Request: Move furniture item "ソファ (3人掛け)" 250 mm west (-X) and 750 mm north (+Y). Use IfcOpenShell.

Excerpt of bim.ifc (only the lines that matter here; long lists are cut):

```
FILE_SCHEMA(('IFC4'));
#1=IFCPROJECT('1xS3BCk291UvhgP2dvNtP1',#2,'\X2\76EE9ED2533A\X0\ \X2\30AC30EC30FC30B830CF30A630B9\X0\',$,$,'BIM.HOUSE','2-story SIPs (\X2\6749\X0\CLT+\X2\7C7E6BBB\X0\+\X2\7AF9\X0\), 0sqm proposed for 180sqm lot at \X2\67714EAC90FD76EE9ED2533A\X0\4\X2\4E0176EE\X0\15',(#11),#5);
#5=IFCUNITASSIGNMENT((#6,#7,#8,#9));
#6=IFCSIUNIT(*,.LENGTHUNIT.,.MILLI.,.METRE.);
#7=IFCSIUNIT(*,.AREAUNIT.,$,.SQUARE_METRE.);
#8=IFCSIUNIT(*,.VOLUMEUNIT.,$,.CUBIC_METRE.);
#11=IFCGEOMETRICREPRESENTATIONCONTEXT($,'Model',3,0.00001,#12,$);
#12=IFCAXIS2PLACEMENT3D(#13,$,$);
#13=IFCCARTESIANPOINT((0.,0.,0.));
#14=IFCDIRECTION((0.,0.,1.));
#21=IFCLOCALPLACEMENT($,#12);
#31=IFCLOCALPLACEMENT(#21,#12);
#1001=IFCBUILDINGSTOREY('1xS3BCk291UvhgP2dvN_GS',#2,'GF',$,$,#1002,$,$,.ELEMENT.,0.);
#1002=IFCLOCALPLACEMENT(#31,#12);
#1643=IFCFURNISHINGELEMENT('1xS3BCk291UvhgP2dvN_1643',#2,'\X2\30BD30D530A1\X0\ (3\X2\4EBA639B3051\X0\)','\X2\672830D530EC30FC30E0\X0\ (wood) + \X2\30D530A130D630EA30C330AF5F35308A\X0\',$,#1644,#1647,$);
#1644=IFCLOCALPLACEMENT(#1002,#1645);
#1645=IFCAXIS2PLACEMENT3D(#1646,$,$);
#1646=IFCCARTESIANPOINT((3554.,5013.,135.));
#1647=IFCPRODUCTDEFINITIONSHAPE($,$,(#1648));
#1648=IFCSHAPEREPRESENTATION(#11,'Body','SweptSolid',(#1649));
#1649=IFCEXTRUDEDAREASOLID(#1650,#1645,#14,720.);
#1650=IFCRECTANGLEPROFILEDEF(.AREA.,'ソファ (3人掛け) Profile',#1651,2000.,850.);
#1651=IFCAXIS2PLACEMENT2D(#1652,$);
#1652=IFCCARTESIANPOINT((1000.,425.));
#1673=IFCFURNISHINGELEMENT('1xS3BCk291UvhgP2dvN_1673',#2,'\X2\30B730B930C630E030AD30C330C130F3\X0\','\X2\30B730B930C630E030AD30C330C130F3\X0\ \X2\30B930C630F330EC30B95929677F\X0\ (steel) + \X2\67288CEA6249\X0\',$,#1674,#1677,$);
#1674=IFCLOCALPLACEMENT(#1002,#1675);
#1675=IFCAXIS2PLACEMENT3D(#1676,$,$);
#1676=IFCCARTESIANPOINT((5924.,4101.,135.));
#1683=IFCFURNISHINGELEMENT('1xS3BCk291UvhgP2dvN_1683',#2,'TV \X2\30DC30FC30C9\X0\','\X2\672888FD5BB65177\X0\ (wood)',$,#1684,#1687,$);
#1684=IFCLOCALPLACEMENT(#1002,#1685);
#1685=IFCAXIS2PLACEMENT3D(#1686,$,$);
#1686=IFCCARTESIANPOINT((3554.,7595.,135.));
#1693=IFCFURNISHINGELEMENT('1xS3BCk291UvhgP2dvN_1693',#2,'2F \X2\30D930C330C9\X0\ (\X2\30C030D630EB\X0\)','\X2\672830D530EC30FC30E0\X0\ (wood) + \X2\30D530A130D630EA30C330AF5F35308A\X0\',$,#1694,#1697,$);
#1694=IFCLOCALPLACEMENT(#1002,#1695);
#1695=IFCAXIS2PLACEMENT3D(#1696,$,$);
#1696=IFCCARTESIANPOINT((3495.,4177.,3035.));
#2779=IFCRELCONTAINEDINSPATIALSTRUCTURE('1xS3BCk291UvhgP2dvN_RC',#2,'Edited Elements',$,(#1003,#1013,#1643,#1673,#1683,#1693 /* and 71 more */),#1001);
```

```python
import ifcopenshell
import ifcopenshell.api.geometry
import ifcopenshell.util.placement
import ifcopenshell.util.unit

model = ifcopenshell.open("bim.ifc")
unit_scale = ifcopenshell.util.unit.calculate_unit_scale(model)

item = model.by_guid("1xS3BCk291UvhgP2dvN_1643")
matrix = ifcopenshell.util.placement.get_local_placement(item.ObjectPlacement)
matrix[0, 3] -= 0.25 / unit_scale
matrix[1, 3] += 0.75 / unit_scale
ifcopenshell.api.geometry.edit_object_placement(model, product=item, matrix=matrix, is_si=False)

print(ifcopenshell.util.placement.get_local_placement(item.ObjectPlacement).round(3) + 0.0)

model.write("bim-out.ifc")
```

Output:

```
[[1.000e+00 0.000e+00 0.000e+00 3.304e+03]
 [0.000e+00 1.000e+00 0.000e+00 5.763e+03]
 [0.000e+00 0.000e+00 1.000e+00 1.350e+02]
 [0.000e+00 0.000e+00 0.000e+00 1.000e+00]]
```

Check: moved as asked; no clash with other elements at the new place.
